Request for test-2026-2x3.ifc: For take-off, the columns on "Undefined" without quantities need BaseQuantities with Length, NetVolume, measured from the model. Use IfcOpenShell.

First a look at what the model holds.

```python
import ifcopenshell
import ifcopenshell.util.element
import ifcopenshell.util.unit

model = ifcopenshell.open("test-2026-2x3.ifc")
print(model.schema)
for unit_type in ("LENGTHUNIT", "AREAUNIT", "VOLUMEUNIT"):
    print(unit_type, ifcopenshell.util.unit.calculate_unit_scale(model, unit_type))
storey = next(s for s in model.by_type("IfcBuildingStorey") if s.Name == "Undefined")
columns = [e for e in ifcopenshell.util.element.get_decomposition(storey) if e.is_a("IfcColumn")]
for e in sorted(columns, key=lambda e: e.id()):
    print(e.id(), e.is_a(), e.Name, list(ifcopenshell.util.element.get_psets(e, qtos_only=True)), sep=" | ")
```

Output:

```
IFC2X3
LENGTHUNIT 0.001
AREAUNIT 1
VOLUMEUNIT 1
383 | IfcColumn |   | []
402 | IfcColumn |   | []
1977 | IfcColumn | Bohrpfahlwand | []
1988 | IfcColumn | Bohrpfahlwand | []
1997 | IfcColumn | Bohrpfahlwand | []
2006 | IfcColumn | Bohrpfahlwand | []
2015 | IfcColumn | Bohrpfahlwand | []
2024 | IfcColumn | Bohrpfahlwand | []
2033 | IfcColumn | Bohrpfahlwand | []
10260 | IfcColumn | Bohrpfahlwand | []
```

```python
import ifcopenshell
import ifcopenshell.api.pset
import ifcopenshell.geom
import ifcopenshell.util.element
import ifcopenshell.util.shape
import ifcopenshell.util.unit

model = ifcopenshell.open("test-2026-2x3.ifc")
unit_scale = ifcopenshell.util.unit.calculate_unit_scale(model)
volume_scale = ifcopenshell.util.unit.calculate_unit_scale(model, "VOLUMEUNIT")
settings = ifcopenshell.geom.settings()

storey = next(s for s in model.by_type("IfcBuildingStorey") if s.Name == "Undefined")
columns = [e for e in ifcopenshell.util.element.get_decomposition(storey) if e.is_a("IfcColumn")]

for e in sorted(columns, key=lambda e: e.id()):
    if ifcopenshell.util.element.get_psets(e, qtos_only=True, should_inherit=False):
        continue
    # Geometry comes back in metres, in the element's own axes.
    shape = ifcopenshell.geom.create_shape(settings, e)
    values = {
        "Length": ifcopenshell.util.shape.get_z(shape.geometry) / unit_scale,
        "NetVolume": ifcopenshell.util.shape.get_volume(shape.geometry) / volume_scale,
    }
    qto = ifcopenshell.api.pset.add_qto(model, product=e, name="BaseQuantities")
    ifcopenshell.api.pset.edit_qto(model, qto=qto, properties=values)
    print(e.id(), {k: round(v, 3) for k, v in values.items()})

model.write("test-2026-2x3_v2.ifc")
```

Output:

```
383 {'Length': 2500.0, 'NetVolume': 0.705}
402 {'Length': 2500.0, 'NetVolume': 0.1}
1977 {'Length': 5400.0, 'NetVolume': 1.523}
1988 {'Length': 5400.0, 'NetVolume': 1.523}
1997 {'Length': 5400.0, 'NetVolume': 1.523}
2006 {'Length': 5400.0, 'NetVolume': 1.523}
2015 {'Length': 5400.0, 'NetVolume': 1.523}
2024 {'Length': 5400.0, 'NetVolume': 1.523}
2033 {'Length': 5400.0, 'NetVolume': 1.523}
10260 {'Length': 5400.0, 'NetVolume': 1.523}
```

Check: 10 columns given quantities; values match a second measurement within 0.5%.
